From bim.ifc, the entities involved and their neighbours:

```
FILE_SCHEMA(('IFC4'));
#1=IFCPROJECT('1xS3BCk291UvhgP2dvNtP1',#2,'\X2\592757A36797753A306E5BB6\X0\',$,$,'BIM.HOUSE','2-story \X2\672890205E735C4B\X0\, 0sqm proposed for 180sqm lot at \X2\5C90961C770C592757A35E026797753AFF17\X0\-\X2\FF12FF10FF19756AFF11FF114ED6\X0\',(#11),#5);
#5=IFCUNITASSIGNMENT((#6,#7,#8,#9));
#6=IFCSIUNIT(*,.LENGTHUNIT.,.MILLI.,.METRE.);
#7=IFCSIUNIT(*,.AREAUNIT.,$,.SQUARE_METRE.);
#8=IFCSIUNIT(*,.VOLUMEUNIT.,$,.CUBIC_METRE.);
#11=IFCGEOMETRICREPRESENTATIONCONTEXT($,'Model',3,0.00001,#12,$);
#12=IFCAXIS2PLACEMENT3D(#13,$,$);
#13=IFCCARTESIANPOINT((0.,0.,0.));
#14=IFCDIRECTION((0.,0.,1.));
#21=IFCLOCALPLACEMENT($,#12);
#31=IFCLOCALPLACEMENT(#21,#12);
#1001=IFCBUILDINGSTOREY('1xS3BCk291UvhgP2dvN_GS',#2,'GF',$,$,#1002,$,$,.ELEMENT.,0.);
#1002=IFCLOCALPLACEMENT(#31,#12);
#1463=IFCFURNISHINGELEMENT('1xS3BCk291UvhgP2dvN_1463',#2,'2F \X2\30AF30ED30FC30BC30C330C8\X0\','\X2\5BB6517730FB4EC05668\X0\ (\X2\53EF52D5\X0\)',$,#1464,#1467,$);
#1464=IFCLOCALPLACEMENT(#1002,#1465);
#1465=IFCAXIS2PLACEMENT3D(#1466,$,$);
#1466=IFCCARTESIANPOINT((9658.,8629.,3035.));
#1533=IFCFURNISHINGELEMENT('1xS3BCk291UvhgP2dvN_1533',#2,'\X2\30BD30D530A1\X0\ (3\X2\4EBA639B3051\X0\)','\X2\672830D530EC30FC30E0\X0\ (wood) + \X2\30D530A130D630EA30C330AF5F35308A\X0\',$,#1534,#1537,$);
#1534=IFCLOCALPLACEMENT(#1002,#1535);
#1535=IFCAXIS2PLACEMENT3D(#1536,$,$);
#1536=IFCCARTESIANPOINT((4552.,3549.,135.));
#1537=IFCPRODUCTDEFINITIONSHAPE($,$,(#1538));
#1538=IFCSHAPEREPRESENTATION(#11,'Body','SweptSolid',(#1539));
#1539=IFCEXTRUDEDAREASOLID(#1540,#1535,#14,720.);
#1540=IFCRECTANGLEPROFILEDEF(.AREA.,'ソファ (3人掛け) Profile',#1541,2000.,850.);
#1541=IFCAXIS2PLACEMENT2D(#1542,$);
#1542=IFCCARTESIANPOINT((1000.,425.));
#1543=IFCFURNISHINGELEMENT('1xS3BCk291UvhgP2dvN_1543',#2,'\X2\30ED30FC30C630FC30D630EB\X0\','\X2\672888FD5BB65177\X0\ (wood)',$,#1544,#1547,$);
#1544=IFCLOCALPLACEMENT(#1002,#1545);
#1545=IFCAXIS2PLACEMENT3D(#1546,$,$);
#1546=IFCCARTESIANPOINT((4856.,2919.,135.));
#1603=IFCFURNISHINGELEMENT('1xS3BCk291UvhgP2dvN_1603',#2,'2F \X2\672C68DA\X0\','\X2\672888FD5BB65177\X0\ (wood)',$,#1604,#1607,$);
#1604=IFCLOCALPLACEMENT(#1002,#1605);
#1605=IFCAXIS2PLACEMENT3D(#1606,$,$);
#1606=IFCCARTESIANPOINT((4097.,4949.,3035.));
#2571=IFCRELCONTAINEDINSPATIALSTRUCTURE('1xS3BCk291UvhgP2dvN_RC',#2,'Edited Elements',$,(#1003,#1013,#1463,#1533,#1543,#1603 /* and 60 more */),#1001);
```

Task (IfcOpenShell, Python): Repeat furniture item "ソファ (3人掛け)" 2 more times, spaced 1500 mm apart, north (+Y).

```python
import numpy as np
import ifcopenshell
import ifcopenshell.api.geometry
import ifcopenshell.api.root
import ifcopenshell.util.element
import ifcopenshell.util.placement

model = ifcopenshell.open("bim.ifc")


def reuse_history(source, copy):
    """copy_class also copies each property set's owner history, people and application; keep the originals."""
    for rel in copy.IsDefinedBy:
        if rel.is_a("IfcRelDefinesByProperties") and (history := rel.RelatingPropertyDefinition.OwnerHistory):
            rel.RelatingPropertyDefinition.OwnerHistory = source.OwnerHistory
            ifcopenshell.util.element.remove_deep2(model, history)


source = model.by_guid("1xS3BCk291UvhgP2dvN_1533")
base = ifcopenshell.util.placement.get_local_placement(source.ObjectPlacement)
step = np.array([0.0, 1.0, 0.0]) * 1500.0

for i in range(1, 3):
    copy = ifcopenshell.api.root.copy_class(model, product=source)
    copy.Representation = ifcopenshell.util.element.copy_deep(
        model, source.Representation, exclude=["IfcGeometricRepresentationContext", "IfcRepresentationMap"]
    )
    reuse_history(source, copy)
    matrix = base.copy()
    matrix[:3, 3] += i * step
    print("added at", matrix[:3, 3].round(3) + 0.0)
    ifcopenshell.api.geometry.edit_object_placement(model, product=copy, matrix=matrix, is_si=False)

model.write("bim-out.ifc")
```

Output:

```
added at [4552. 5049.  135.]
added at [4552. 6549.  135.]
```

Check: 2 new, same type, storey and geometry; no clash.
